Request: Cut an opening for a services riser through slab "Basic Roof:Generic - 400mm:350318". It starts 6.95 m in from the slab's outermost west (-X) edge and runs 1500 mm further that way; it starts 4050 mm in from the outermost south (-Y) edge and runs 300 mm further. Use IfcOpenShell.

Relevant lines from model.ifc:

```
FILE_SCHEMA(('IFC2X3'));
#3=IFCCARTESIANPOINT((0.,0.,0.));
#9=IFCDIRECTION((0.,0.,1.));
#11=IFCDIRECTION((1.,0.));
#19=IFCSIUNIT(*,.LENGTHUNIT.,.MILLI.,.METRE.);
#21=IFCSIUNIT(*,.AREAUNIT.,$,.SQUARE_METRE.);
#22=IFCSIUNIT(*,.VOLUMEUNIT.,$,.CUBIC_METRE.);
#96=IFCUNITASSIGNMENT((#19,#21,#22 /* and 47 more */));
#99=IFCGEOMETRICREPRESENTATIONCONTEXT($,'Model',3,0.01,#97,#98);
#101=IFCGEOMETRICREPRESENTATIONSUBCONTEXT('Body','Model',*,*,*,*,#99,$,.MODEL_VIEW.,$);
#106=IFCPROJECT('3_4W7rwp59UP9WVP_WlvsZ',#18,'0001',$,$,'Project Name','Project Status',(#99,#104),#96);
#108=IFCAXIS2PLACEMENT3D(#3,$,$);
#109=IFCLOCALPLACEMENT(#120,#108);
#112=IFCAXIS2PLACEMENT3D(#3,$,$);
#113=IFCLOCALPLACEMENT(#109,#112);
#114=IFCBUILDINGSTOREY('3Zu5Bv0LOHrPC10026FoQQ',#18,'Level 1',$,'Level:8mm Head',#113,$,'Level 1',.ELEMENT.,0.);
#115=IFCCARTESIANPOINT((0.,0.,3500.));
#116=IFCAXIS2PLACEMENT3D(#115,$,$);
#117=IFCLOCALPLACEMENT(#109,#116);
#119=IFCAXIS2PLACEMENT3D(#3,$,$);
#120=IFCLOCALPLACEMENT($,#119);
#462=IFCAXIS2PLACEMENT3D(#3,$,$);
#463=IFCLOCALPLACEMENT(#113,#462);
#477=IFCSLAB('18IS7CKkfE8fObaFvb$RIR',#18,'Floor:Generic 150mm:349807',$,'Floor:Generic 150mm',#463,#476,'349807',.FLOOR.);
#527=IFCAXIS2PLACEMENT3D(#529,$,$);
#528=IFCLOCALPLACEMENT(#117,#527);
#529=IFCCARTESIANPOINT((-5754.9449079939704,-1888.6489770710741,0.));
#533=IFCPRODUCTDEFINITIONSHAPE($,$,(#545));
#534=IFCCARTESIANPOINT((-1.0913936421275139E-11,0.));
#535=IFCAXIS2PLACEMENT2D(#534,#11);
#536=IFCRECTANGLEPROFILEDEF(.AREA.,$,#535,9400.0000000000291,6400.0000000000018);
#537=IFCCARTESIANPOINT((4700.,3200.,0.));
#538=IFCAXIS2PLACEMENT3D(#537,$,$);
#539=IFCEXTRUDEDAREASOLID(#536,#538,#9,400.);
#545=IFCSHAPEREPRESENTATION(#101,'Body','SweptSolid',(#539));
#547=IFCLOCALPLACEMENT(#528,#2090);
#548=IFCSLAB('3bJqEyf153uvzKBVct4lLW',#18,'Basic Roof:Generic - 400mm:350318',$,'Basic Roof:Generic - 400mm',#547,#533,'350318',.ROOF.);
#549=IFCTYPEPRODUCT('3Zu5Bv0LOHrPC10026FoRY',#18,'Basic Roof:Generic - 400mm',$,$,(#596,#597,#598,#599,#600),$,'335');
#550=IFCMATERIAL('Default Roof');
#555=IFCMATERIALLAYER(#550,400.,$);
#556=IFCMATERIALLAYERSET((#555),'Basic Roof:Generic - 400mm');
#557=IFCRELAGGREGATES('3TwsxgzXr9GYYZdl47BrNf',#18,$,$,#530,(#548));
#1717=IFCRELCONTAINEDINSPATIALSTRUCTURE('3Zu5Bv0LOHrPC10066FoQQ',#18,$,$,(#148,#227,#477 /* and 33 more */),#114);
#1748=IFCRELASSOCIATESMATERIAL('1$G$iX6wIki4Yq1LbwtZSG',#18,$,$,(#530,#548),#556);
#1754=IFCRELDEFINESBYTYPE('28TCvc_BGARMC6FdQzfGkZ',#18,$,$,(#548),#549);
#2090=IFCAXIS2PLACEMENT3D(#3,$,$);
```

```python
import numpy as np
import ifcopenshell
import ifcopenshell.api.feature
import ifcopenshell.api.geometry
import ifcopenshell.api.root
import ifcopenshell.geom
import ifcopenshell.util.placement
import ifcopenshell.util.representation
import ifcopenshell.util.shape
import ifcopenshell.util.unit

model = ifcopenshell.open("model.ifc")
unit_scale = ifcopenshell.util.unit.calculate_unit_scale(model)
settings = ifcopenshell.geom.settings()


def volume(element):
    """Net volume in cubic metres, openings subtracted."""
    shape = ifcopenshell.geom.create_shape(settings, element)
    return ifcopenshell.util.shape.get_volume(shape.geometry)


slab = model.by_guid("3bJqEyf153uvzKBVct4lLW")
before = volume(slab)

# Extent in the slab's own axes, in metres. The edges named are its -X and -Y sides.
slab_shape = ifcopenshell.geom.create_shape(settings, slab)
vertices = ifcopenshell.util.shape.get_vertices(slab_shape.geometry)
x_min, y_min, bottom = vertices.min(axis=0)
top = vertices[:, 2].max()

opening = ifcopenshell.api.root.create_entity(model, ifc_class="IfcOpeningElement", name="Services riser opening")
context = ifcopenshell.util.representation.get_context(model, "Model", "Body", "MODEL_VIEW")
width, depth = 1.5, 0.3
outline = [(0.0, 0.0), (width, 0.0), (width, depth), (0.0, depth), (0.0, 0.0)]
# Overshoot both faces by 50 mm so the cut is clean.
shape = ifcopenshell.api.geometry.add_slab_representation(
    model, context=context, depth=top - bottom + 0.1, polyline=outline
)
ifcopenshell.api.geometry.assign_representation(model, product=opening, representation=shape)

matrix = ifcopenshell.util.placement.get_local_placement(slab.ObjectPlacement)
matrix[:, 3] = matrix @ np.append(np.array([x_min + 6.95, y_min + 4.05, bottom - 0.05]) / unit_scale, 1.0)
ifcopenshell.api.geometry.edit_object_placement(model, product=opening, matrix=matrix, is_si=False)
ifcopenshell.api.feature.add_feature(model, feature=opening, element=slab)

after = volume(slab)

print(f"slab volume {before:.3f} -> {after:.3f} m3")

model.write("model_rev.ifc")
```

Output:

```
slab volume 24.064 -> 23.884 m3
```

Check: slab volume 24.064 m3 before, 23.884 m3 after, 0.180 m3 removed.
